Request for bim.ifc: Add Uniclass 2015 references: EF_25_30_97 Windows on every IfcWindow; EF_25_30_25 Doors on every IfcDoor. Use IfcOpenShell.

First a look at what the model holds.

```python
import ifcopenshell

model = ifcopenshell.open("bim.ifc")
print(model.schema)
print("classifications:", [c.Name for c in model.by_type("IfcClassification")])
for ifc_class in ("IfcDoor", "IfcRoof", "IfcStair", "IfcWall", "IfcWindow"):
    print(ifc_class, len(model.by_type(ifc_class)))
```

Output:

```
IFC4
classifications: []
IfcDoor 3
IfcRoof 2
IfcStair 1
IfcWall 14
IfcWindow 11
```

```python
import ifcopenshell
import ifcopenshell.api.classification

model = ifcopenshell.open("bim.ifc")

system = ifcopenshell.api.classification.add_classification(model, classification="Uniclass 2015")

codes = {
    "IfcWindow": ("EF_25_30_97", "Windows"),
    "IfcDoor": ("EF_25_30_25", "Doors"),
}
for ifc_class, (code, name) in codes.items():
    products = model.by_type(ifc_class)
    ifcopenshell.api.classification.add_reference(
        model, products=products, classification=system, identification=code, name=name
    )
    print(code, len(products))

model.write("bim_rev.ifc")
```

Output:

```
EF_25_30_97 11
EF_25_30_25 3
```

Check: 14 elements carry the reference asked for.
